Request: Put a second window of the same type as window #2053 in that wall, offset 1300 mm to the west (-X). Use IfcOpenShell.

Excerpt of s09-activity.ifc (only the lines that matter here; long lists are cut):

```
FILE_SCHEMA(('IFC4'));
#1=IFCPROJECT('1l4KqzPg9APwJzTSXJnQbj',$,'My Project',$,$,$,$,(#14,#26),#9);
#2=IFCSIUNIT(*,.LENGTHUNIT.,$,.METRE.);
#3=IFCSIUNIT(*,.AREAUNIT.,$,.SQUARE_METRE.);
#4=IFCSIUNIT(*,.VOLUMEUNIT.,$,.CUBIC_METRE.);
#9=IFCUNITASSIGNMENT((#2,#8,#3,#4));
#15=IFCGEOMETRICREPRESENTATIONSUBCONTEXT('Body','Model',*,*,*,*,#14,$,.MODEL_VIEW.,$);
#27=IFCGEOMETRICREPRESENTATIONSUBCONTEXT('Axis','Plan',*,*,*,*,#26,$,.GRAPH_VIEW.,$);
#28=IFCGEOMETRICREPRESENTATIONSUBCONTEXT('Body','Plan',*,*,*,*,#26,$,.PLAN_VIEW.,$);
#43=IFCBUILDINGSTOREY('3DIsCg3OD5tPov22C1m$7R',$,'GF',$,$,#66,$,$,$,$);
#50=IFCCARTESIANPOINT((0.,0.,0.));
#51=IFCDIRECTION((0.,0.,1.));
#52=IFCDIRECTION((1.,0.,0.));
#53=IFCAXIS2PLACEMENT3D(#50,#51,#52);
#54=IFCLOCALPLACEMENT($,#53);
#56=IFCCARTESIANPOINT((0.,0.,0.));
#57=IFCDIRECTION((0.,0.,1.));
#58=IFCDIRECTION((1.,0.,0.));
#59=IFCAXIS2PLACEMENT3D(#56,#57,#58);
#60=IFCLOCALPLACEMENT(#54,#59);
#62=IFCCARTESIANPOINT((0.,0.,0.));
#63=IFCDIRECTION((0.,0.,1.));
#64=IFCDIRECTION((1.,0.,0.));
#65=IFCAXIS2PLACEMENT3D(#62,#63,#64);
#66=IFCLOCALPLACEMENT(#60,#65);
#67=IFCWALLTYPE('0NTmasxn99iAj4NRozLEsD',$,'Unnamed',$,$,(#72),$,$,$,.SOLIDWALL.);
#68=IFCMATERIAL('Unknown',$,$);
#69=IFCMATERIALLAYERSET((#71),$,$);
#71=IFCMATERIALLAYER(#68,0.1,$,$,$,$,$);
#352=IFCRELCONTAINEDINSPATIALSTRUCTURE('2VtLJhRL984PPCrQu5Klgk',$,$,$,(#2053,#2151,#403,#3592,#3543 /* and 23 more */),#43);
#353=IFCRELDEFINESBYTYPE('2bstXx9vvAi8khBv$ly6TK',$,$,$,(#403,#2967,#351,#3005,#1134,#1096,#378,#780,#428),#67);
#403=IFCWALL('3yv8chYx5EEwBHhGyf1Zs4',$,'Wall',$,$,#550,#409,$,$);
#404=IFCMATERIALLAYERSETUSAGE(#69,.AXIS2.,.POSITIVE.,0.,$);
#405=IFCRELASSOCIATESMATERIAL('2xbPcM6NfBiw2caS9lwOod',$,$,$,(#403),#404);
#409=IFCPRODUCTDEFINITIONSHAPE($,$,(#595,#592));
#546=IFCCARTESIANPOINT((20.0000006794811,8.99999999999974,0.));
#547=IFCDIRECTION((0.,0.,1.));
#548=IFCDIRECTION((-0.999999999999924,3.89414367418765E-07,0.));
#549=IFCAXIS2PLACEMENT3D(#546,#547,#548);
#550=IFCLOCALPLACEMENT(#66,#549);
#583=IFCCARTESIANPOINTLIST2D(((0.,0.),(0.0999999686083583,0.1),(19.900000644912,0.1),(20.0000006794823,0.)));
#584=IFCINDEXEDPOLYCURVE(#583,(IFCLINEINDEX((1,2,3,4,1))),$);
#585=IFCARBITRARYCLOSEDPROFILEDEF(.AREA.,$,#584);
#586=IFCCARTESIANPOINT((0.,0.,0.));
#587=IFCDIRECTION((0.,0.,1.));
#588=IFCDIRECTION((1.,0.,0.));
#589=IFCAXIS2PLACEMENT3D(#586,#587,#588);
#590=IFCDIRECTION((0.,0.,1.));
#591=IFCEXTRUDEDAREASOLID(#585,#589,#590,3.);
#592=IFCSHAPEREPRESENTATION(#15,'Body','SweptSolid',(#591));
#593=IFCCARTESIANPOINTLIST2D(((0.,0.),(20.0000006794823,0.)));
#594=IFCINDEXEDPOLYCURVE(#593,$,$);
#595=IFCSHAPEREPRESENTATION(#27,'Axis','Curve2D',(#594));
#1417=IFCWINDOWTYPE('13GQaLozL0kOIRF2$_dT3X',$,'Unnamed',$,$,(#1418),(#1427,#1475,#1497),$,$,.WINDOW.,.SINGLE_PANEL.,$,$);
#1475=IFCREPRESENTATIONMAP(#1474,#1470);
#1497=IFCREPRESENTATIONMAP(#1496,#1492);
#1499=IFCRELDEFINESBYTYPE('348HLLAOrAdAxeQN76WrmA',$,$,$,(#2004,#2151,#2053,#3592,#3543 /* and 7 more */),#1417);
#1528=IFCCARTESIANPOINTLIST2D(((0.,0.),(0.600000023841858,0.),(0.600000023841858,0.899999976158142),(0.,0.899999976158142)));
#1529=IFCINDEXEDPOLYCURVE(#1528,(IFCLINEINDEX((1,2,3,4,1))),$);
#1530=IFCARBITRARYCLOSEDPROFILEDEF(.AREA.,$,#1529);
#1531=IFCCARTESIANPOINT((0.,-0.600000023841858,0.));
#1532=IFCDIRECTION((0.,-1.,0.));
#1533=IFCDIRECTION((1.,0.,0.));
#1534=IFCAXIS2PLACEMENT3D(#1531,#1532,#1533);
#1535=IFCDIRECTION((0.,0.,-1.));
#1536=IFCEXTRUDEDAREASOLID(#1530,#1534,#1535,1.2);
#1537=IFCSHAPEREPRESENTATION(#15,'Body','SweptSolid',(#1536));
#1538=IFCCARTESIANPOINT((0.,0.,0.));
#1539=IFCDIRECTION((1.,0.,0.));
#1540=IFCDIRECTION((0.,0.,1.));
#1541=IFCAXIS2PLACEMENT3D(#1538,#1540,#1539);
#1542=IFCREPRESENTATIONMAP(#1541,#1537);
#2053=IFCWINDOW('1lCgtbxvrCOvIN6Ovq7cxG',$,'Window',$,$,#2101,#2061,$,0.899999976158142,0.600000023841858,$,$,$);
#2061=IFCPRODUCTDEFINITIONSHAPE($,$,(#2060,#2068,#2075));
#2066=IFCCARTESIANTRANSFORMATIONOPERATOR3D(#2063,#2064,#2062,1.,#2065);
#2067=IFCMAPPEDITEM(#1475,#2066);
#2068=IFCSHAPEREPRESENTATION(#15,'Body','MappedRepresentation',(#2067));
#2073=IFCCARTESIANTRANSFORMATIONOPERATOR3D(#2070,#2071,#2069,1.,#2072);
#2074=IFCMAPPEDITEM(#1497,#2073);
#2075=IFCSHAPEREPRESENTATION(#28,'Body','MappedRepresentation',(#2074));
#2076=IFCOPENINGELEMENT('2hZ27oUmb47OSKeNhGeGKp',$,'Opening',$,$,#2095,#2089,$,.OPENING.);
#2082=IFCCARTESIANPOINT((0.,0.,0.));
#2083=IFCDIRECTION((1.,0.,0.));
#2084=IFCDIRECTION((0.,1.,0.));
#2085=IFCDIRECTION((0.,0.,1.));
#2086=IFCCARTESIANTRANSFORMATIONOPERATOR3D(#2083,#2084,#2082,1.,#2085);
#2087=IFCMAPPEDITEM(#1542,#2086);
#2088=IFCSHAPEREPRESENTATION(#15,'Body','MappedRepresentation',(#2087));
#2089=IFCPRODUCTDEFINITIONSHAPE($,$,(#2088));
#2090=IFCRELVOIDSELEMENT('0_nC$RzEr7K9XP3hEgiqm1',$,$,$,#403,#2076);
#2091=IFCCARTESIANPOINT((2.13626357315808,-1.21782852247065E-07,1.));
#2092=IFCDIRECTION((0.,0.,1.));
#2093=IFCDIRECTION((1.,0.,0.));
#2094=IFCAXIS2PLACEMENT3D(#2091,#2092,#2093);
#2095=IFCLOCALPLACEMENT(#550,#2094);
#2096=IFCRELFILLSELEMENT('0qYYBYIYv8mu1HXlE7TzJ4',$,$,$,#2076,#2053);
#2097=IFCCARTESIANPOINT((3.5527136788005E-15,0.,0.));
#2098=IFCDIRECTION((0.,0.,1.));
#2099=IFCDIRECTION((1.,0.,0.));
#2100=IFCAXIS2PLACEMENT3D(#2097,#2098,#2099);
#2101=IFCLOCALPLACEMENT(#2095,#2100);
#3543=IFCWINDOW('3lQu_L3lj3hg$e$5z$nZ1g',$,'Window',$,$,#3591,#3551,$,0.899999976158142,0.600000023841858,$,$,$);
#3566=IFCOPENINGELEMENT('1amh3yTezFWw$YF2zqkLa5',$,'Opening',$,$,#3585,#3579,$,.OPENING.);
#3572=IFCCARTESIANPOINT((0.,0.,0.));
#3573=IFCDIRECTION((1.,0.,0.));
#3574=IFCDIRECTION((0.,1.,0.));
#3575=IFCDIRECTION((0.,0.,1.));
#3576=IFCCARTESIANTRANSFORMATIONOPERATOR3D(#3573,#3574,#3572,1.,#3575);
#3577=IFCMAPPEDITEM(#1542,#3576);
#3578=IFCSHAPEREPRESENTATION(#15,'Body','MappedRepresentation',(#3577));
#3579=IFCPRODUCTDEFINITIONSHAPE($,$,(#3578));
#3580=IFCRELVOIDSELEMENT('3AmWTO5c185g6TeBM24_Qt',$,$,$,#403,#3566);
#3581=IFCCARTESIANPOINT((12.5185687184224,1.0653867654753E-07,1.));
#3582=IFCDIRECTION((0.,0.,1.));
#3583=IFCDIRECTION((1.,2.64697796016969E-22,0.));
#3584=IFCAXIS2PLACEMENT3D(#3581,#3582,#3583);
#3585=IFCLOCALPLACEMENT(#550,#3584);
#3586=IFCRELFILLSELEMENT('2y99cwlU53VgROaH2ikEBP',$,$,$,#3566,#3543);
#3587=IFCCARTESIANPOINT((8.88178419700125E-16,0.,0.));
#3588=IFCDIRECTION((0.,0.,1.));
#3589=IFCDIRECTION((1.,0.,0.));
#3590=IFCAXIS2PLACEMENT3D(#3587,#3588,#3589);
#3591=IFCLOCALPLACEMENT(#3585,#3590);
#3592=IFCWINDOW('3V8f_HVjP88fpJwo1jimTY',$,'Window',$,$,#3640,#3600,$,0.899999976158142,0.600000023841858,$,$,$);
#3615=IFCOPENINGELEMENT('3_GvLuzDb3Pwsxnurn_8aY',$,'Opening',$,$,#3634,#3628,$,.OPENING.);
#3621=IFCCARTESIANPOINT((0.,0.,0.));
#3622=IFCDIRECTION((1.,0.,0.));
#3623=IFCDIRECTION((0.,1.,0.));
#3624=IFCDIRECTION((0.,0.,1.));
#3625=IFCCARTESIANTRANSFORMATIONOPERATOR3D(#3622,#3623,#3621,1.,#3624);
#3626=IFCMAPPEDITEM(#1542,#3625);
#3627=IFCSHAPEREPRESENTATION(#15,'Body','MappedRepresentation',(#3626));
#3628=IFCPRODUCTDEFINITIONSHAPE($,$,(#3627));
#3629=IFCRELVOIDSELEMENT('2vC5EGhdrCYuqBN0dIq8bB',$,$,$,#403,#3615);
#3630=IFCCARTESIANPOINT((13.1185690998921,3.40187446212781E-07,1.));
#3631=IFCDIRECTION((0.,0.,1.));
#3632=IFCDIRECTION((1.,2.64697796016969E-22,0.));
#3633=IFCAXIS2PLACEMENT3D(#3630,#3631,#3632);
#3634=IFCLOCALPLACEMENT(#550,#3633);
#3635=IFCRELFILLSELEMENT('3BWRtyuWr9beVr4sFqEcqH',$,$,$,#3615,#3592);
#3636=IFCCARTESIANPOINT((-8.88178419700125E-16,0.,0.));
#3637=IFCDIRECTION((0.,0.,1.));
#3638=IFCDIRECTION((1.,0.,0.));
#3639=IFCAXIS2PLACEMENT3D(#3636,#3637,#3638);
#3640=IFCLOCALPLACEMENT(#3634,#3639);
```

```python
import ifcopenshell
import ifcopenshell.api.feature
import ifcopenshell.api.geometry
import ifcopenshell.api.root
import ifcopenshell.geom
import ifcopenshell.util.element
import ifcopenshell.util.placement
import ifcopenshell.util.shape

model = ifcopenshell.open("s09-activity.ifc")
settings = ifcopenshell.geom.settings()


def volume(element):
    """Net volume in cubic metres, openings subtracted."""
    shape = ifcopenshell.geom.create_shape(settings, element)
    return ifcopenshell.util.shape.get_volume(shape.geometry)


window = model.by_id(2053)
opening = window.FillsVoids[0].RelatingOpeningElement
wall = opening.VoidsElements[0].RelatingBuildingElement
before = volume(wall)
shift = ifcopenshell.util.placement.get_local_placement(wall.ObjectPlacement)[:3, 0] * 1.3

# copy_class copies the void relationship, type, container and properties, but no geometry.
new_opening = ifcopenshell.api.root.copy_class(model, product=opening)
new_opening.Representation = ifcopenshell.util.element.copy_deep(
    model, opening.Representation, exclude=["IfcGeometricRepresentationContext", "IfcRepresentationMap"]
)
new_window = ifcopenshell.api.root.copy_class(model, product=window)
new_window.Representation = ifcopenshell.util.element.copy_deep(
    model, window.Representation, exclude=["IfcGeometricRepresentationContext", "IfcRepresentationMap"]
)
ifcopenshell.api.feature.add_filling(model, opening=new_opening, element=new_window)

for old, new in ((opening, new_opening), (window, new_window)):
    matrix = ifcopenshell.util.placement.get_local_placement(old.ObjectPlacement)
    matrix[:3, 3] += shift
    ifcopenshell.api.geometry.edit_object_placement(model, product=new, matrix=matrix, is_si=False)

after = volume(wall)

print(f"wall volume {before:.3f} -> {after:.3f} m3")

model.write("s09-activity_rev.ifc")
```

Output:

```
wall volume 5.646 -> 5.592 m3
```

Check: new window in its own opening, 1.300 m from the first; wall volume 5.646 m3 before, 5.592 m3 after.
